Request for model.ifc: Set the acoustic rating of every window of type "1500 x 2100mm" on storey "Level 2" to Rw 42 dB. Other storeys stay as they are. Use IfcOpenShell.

First a look at what the model holds.

```python
import ifcopenshell
import ifcopenshell.util.element

model = ifcopenshell.open("model.ifc")
print(model.schema)
storey = next(s for s in model.by_type("IfcBuildingStorey") if s.Name == "Level 2")
windows = [e for e in ifcopenshell.util.element.get_decomposition(storey) if e.is_a("IfcWindow")]
seen = {}
for e in windows:
    element_type = ifcopenshell.util.element.get_type(e)
    key = (element_type.Name if element_type != e and element_type else None, ifcopenshell.util.element.get_pset(e, "Pset_WindowCommon", "AcousticRating"))
    seen[key] = seen.get(key, 0) + 1
for (name, value), count in sorted(seen.items(), key=str):
    print(count, "x", name, "|", value)
```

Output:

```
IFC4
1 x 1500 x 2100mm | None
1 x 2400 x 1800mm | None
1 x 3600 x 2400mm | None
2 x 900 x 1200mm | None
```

```python
import ifcopenshell
import ifcopenshell.api.pset
import ifcopenshell.util.element

model = ifcopenshell.open("model.ifc")

storey = next(s for s in model.by_type("IfcBuildingStorey") if s.Name == "Level 2")
windows = [e for e in ifcopenshell.util.element.get_decomposition(storey) if e.is_a("IfcWindow")]

count = 0
for e in windows:
    element_type = ifcopenshell.util.element.get_type(e)
    if element_type in (None, e) or element_type.Name != "1500 x 2100mm":
        continue
    # add_pset returns the element's existing set when there is one.
    pset = ifcopenshell.api.pset.add_pset(model, product=e, name="Pset_WindowCommon")
    ifcopenshell.api.pset.edit_pset(model, pset=pset, properties={"AcousticRating": "Rw 42 dB"})
    count += 1

print(count, "windows updated")

model.write("model_edited.ifc")
```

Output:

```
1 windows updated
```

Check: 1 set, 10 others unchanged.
